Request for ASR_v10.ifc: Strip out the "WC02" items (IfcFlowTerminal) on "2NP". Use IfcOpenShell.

First a look at what the model holds.

```python
import ifcopenshell
import ifcopenshell.util.element

model = ifcopenshell.open("ASR_v10.ifc")
print(model.schema)
storey = next(s for s in model.by_type("IfcBuildingStorey") if s.Name == "2NP")
terminals = [e for e in ifcopenshell.util.element.get_decomposition(storey) if e.is_a("IfcFlowTerminal")]
seen = {}
for e in terminals:
    element_type = ifcopenshell.util.element.get_type(e)
    name = element_type.Name if element_type not in (None, e) else None
    seen[name] = seen.get(name, 0) + 1
for name, count in sorted(seen.items(), key=str):
    print(count, "x", name)
```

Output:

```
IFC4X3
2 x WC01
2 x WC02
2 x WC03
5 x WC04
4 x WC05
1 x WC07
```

```python
import ifcopenshell
import ifcopenshell.api.root
import ifcopenshell.util.element

model = ifcopenshell.open("ASR_v10.ifc")

storey = next(s for s in model.by_type("IfcBuildingStorey") if s.Name == "2NP")
terminals = [e for e in ifcopenshell.util.element.get_decomposition(storey) if e.is_a("IfcFlowTerminal")]
targets = [e for e in terminals if (t := ifcopenshell.util.element.get_type(e)) not in (None, e) and t.Name == "WC02"]

for e in targets:
    ifcopenshell.api.root.remove_product(model, product=e)
print(len(targets), "removed")

model.write("ASR_v10_rev.ifc")
```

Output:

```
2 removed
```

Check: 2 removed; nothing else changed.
